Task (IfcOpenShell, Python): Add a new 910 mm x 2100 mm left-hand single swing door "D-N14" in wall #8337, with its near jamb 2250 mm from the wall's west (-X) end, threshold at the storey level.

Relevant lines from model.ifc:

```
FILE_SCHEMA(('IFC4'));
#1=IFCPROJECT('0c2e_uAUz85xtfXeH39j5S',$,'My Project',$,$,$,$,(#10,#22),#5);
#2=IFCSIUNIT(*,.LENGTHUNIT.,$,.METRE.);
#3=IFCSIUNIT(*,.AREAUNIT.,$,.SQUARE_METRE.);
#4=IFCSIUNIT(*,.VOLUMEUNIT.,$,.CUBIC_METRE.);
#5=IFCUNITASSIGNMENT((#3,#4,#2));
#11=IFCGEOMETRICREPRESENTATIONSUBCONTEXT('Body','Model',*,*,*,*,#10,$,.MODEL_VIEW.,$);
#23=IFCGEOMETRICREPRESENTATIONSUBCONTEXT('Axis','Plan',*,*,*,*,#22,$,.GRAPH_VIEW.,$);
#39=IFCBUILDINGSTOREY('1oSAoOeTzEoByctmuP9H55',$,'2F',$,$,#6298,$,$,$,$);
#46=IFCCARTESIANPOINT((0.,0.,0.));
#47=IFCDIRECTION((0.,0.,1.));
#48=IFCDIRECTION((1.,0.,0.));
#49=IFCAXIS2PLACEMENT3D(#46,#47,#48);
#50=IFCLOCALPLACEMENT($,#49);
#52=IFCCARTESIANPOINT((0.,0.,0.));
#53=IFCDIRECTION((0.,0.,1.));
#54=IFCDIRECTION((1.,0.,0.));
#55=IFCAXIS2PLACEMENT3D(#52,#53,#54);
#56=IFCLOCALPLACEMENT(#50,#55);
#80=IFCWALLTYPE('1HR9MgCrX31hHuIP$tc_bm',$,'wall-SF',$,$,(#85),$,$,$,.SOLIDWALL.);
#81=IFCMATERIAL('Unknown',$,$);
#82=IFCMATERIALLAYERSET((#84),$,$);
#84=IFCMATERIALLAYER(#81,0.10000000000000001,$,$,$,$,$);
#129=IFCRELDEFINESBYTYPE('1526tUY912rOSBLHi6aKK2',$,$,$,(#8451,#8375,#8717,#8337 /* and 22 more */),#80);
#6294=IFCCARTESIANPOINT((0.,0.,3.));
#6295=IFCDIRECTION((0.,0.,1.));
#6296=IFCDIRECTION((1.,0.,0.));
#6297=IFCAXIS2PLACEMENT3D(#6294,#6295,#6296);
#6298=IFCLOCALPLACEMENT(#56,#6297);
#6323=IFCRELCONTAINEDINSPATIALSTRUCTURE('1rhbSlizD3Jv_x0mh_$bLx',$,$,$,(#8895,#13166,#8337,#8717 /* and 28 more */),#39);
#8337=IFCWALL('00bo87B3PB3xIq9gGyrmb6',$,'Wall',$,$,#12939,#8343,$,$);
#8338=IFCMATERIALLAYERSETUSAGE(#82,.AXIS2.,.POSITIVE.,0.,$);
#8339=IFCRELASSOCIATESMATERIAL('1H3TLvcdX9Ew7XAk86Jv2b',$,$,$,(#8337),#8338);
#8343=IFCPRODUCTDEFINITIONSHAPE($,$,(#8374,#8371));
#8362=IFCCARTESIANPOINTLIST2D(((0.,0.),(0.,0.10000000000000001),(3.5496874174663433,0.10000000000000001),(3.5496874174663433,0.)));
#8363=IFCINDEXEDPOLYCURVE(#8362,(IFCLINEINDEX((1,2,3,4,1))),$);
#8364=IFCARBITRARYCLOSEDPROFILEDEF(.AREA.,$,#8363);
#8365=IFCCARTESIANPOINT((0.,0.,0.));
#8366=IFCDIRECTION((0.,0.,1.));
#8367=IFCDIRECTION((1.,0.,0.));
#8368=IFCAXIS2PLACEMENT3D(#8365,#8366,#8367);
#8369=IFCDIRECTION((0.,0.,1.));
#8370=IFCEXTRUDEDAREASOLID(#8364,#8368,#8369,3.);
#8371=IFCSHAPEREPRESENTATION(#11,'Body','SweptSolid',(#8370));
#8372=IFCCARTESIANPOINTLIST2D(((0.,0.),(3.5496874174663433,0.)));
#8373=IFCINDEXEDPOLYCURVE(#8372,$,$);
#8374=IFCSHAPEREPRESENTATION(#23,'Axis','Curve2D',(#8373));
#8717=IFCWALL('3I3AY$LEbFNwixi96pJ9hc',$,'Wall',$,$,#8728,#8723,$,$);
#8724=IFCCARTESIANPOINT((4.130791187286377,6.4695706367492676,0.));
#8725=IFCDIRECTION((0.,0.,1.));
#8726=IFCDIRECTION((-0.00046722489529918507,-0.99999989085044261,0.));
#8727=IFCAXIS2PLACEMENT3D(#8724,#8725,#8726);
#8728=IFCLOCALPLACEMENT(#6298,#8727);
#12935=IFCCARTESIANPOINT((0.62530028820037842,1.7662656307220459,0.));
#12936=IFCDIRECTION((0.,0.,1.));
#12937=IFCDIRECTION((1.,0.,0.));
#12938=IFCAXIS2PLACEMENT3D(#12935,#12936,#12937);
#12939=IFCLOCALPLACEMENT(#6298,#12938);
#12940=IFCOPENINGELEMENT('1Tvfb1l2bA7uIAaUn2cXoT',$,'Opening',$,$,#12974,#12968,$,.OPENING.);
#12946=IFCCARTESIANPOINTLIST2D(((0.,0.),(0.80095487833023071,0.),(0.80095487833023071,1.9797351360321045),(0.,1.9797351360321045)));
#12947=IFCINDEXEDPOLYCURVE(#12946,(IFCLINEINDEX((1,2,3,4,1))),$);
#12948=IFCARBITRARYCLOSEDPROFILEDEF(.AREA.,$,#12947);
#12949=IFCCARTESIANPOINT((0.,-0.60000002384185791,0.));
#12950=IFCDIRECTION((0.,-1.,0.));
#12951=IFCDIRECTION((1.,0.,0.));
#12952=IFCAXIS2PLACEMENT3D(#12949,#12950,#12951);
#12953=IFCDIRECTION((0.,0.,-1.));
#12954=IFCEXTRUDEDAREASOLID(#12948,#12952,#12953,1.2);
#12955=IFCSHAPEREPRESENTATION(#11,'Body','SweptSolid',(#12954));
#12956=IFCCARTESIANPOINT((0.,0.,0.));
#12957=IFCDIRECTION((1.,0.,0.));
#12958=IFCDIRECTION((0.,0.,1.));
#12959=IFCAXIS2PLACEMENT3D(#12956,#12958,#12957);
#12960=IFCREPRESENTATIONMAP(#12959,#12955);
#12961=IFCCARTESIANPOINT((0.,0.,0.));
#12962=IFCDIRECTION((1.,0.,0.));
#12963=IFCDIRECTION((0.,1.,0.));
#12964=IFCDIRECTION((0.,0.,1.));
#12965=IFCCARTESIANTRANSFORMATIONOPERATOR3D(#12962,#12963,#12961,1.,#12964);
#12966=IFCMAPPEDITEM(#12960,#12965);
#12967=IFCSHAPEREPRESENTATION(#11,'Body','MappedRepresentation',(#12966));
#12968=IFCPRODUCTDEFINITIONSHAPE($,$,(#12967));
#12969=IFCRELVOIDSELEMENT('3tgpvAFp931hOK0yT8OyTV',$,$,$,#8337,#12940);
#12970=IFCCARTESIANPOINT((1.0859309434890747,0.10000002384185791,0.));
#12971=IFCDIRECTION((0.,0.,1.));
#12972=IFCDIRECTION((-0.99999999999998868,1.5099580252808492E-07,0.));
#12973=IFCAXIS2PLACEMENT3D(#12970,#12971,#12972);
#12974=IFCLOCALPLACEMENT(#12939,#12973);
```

```python
import numpy as np
import ifcopenshell
import ifcopenshell.api.feature
import ifcopenshell.api.geometry
import ifcopenshell.api.root
import ifcopenshell.api.spatial
import ifcopenshell.geom
import ifcopenshell.util.element
import ifcopenshell.util.placement
import ifcopenshell.util.representation
import ifcopenshell.util.shape
import ifcopenshell.util.unit

model = ifcopenshell.open("model.ifc")
unit_scale = ifcopenshell.util.unit.calculate_unit_scale(model)
settings = ifcopenshell.geom.settings()


def volume(element):
    """Net volume in cubic metres, openings subtracted."""
    shape = ifcopenshell.geom.create_shape(settings, element)
    return ifcopenshell.util.shape.get_volume(shape.geometry)


wall = model.by_guid("00bo87B3PB3xIq9gGyrmb6")
storey = ifcopenshell.util.element.get_container(wall, ifc_class="IfcBuildingStorey")
context = ifcopenshell.util.representation.get_context(model, "Model", "Body", "MODEL_VIEW")
before = volume(wall)

width, height, from_end, sill = 0.91, 2.1, 2.25, 0.0  # metres

# The wall runs along its own X axis, and the end named is its -X end.
wall_shape = ifcopenshell.geom.create_shape(settings, wall)
x, y, z = ifcopenshell.util.shape.get_vertices(wall_shape.geometry).T
start = x.min() + from_end
face, thickness = float(y.min()), float(y.max() - y.min())
wall_matrix = ifcopenshell.util.placement.get_local_placement(wall.ObjectPlacement)
level = ifcopenshell.util.placement.get_local_placement(storey.ObjectPlacement)[2, 3]


def in_wall(x, y):
    """Placement at x, y metres in the wall's axes, at sill height."""
    matrix = wall_matrix.copy()
    matrix[:, 3] = wall_matrix @ np.array([x / unit_scale, y / unit_scale, 0.0, 1.0])
    matrix[2, 3] = level + sill / unit_scale
    return matrix


# Opening: a box that overshoots both wall faces by 50 mm.
opening = ifcopenshell.api.root.create_entity(model, ifc_class="IfcOpeningElement", predefined_type="OPENING")
box = ifcopenshell.api.geometry.add_wall_representation(
    model, context=context, length=width, height=height, thickness=thickness + 0.1
)
ifcopenshell.api.geometry.assign_representation(model, product=opening, representation=box)
ifcopenshell.api.geometry.edit_object_placement(model, product=opening, matrix=in_wall(start, face - 0.05), is_si=False)
ifcopenshell.api.feature.add_feature(model, feature=opening, element=wall)

door = ifcopenshell.api.root.create_entity(model, ifc_class="IfcDoor", name="D-N14", predefined_type="DOOR")
door.OverallWidth, door.OverallHeight = width / unit_scale, height / unit_scale
door.OperationType = "SINGLE_SWING_LEFT"
body = ifcopenshell.api.geometry.add_door_representation(
    model,
    context=context,
    overall_width=door.OverallWidth,
    overall_height=door.OverallHeight,
    operation_type="SINGLE_SWING_LEFT",
    lining_properties={"LiningDepth": thickness / unit_scale, "ThresholdDepth": thickness / unit_scale},
)
ifcopenshell.api.geometry.assign_representation(model, product=door, representation=body)
ifcopenshell.api.spatial.assign_container(model, products=[door], relating_structure=storey)
ifcopenshell.api.feature.add_filling(model, opening=opening, element=door)

# The lining spans the wall, so the door starts at the wall face.
ifcopenshell.api.geometry.edit_object_placement(model, product=door, matrix=in_wall(start, face), is_si=False)

after = volume(wall)

print(f"wall volume {before:.3f} -> {after:.3f} m3")

model.write("model-out.ifc")
```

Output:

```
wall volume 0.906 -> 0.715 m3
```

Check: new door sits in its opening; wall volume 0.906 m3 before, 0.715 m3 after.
